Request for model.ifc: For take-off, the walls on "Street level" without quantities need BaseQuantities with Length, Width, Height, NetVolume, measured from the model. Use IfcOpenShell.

First a look at what the model holds.

```python
import ifcopenshell
import ifcopenshell.util.element
import ifcopenshell.util.unit

model = ifcopenshell.open("model.ifc")
print(model.schema)
for unit_type in ("LENGTHUNIT", "AREAUNIT", "VOLUMEUNIT"):
    print(unit_type, ifcopenshell.util.unit.calculate_unit_scale(model, unit_type))
storey = next(s for s in model.by_type("IfcBuildingStorey") if s.Name == "Street level")
walls = [e for e in ifcopenshell.util.element.get_decomposition(storey) if e.is_a("IfcWall")]
for e in sorted(walls, key=lambda e: e.id()):
    print(e.id(), e.is_a(), e.Name, list(ifcopenshell.util.element.get_psets(e, qtos_only=True)), sep=" | ")
```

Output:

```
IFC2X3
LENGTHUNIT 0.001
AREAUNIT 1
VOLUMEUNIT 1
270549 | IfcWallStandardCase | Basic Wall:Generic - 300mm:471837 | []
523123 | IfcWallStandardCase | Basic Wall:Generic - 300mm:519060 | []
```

```python
import ifcopenshell
import ifcopenshell.api.pset
import ifcopenshell.geom
import ifcopenshell.util.element
import ifcopenshell.util.shape
import ifcopenshell.util.unit

model = ifcopenshell.open("model.ifc")
unit_scale = ifcopenshell.util.unit.calculate_unit_scale(model)
volume_scale = ifcopenshell.util.unit.calculate_unit_scale(model, "VOLUMEUNIT")
settings = ifcopenshell.geom.settings()

storey = next(s for s in model.by_type("IfcBuildingStorey") if s.Name == "Street level")
walls = [e for e in ifcopenshell.util.element.get_decomposition(storey) if e.is_a("IfcWall")]

for e in sorted(walls, key=lambda e: e.id()):
    if ifcopenshell.util.element.get_psets(e, qtos_only=True, should_inherit=False):
        continue
    # Geometry comes back in metres, in the element's own axes.
    shape = ifcopenshell.geom.create_shape(settings, e)
    values = {
        "Length": ifcopenshell.util.shape.get_x(shape.geometry) / unit_scale,
        "Width": ifcopenshell.util.shape.get_y(shape.geometry) / unit_scale,
        "Height": ifcopenshell.util.shape.get_z(shape.geometry) / unit_scale,
        "NetVolume": ifcopenshell.util.shape.get_volume(shape.geometry) / volume_scale,
    }
    qto = ifcopenshell.api.pset.add_qto(model, product=e, name="BaseQuantities")
    ifcopenshell.api.pset.edit_qto(model, qto=qto, properties=values)
    print(e.id(), {k: round(v, 3) for k, v in values.items()})

model.write("model-out.ifc")
```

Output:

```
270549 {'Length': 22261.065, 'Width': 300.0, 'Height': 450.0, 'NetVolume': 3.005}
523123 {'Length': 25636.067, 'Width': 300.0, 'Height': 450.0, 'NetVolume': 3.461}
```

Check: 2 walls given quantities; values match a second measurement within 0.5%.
